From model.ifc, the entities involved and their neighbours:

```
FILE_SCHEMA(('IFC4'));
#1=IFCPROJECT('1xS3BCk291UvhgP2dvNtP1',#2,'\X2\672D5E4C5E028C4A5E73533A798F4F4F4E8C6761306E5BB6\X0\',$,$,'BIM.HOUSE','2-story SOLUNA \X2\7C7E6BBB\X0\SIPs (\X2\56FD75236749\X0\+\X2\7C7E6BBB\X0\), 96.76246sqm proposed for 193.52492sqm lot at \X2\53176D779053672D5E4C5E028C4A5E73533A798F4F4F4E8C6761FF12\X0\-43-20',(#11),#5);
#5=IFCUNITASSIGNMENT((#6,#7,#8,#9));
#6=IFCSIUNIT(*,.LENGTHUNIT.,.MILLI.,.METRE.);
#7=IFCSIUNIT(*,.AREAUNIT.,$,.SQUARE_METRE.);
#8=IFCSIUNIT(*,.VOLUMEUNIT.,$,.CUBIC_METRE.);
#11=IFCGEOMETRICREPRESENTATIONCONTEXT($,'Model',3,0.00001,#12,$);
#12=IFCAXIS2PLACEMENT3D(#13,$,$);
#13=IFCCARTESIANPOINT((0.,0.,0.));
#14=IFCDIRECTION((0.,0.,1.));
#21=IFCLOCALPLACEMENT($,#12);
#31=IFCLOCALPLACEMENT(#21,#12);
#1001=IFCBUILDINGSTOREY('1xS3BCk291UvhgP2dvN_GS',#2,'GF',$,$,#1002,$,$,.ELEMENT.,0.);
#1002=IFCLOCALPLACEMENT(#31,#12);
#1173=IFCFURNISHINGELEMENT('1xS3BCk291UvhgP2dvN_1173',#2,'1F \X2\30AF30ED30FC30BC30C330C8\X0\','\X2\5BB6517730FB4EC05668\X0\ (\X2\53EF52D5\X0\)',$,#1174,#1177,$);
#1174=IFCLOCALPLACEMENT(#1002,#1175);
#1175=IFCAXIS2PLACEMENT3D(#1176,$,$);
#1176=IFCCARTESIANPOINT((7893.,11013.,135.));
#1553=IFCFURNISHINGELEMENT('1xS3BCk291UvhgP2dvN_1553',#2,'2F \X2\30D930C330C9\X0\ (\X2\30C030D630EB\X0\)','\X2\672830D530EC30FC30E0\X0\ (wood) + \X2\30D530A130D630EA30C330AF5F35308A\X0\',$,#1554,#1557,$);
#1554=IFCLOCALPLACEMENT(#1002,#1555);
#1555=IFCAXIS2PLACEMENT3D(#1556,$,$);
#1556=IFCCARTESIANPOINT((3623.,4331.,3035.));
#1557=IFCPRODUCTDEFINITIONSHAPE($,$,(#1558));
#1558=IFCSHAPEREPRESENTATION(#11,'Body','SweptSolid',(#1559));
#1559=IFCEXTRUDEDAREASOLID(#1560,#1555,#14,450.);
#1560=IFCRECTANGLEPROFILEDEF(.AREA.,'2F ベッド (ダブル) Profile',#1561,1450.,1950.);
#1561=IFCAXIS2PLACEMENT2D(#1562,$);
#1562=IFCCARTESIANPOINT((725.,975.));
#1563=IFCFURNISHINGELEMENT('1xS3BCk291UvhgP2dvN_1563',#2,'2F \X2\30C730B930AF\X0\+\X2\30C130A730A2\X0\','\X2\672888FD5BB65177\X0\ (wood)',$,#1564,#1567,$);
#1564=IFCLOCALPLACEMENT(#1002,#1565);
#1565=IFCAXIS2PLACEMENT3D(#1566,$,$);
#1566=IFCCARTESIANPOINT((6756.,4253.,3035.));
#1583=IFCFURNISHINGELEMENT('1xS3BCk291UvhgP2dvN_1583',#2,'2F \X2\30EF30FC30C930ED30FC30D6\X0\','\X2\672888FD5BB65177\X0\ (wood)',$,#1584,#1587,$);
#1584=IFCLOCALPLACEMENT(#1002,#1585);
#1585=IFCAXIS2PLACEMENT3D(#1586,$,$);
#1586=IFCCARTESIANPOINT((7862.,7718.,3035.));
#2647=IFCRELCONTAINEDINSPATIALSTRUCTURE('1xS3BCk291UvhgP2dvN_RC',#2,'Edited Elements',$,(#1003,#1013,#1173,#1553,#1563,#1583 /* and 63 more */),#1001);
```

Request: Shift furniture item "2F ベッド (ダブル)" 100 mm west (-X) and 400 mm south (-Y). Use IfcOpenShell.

```python
import ifcopenshell
import ifcopenshell.api.geometry
import ifcopenshell.util.placement

model = ifcopenshell.open("model.ifc")

item = model.by_guid("1xS3BCk291UvhgP2dvN_1553")
matrix = ifcopenshell.util.placement.get_local_placement(item.ObjectPlacement)
matrix[0, 3] -= 100.0
matrix[1, 3] -= 400.0
ifcopenshell.api.geometry.edit_object_placement(model, product=item, matrix=matrix, is_si=False)

print(ifcopenshell.util.placement.get_local_placement(item.ObjectPlacement).round(3) + 0.0)

model.write("model_rev.ifc")
```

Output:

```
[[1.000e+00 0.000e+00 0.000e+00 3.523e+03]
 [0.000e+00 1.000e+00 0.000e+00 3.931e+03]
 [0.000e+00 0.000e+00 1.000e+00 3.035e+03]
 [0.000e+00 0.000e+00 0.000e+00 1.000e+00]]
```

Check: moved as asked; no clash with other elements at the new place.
